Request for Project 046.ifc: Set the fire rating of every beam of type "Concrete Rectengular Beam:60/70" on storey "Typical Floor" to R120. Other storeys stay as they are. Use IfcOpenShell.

First a look at what the model holds.

```python
import ifcopenshell
import ifcopenshell.util.element

model = ifcopenshell.open("Project 046.ifc")
print(model.schema)
storey = next(s for s in model.by_type("IfcBuildingStorey") if s.Name == "Typical Floor")
beams = [e for e in ifcopenshell.util.element.get_decomposition(storey) if e.is_a("IfcBeam")]
seen = {}
for e in beams:
    element_type = ifcopenshell.util.element.get_type(e)
    key = (element_type.Name if element_type != e and element_type else None, ifcopenshell.util.element.get_pset(e, "Pset_BeamCommon", "FireRating"))
    seen[key] = seen.get(key, 0) + 1
for (name, value), count in sorted(seen.items(), key=str):
    print(count, "x", name, "|", value)
```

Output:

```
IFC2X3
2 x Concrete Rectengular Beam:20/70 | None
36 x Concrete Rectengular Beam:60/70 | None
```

```python
import ifcopenshell
import ifcopenshell.api.pset
import ifcopenshell.util.element

model = ifcopenshell.open("Project 046.ifc")

storey = next(s for s in model.by_type("IfcBuildingStorey") if s.Name == "Typical Floor")
beams = [e for e in ifcopenshell.util.element.get_decomposition(storey) if e.is_a("IfcBeam")]

count = 0
for e in beams:
    element_type = ifcopenshell.util.element.get_type(e)
    if element_type in (None, e) or element_type.Name != "Concrete Rectengular Beam:60/70":
        continue
    # add_pset returns the element's existing set when there is one.
    pset = ifcopenshell.api.pset.add_pset(model, product=e, name="Pset_BeamCommon")
    ifcopenshell.api.pset.edit_pset(model, pset=pset, properties={"FireRating": "R120"})
    count += 1

print(count, "beams updated")

model.write("Project 046_v2.ifc")
```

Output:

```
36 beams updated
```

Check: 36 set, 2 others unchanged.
